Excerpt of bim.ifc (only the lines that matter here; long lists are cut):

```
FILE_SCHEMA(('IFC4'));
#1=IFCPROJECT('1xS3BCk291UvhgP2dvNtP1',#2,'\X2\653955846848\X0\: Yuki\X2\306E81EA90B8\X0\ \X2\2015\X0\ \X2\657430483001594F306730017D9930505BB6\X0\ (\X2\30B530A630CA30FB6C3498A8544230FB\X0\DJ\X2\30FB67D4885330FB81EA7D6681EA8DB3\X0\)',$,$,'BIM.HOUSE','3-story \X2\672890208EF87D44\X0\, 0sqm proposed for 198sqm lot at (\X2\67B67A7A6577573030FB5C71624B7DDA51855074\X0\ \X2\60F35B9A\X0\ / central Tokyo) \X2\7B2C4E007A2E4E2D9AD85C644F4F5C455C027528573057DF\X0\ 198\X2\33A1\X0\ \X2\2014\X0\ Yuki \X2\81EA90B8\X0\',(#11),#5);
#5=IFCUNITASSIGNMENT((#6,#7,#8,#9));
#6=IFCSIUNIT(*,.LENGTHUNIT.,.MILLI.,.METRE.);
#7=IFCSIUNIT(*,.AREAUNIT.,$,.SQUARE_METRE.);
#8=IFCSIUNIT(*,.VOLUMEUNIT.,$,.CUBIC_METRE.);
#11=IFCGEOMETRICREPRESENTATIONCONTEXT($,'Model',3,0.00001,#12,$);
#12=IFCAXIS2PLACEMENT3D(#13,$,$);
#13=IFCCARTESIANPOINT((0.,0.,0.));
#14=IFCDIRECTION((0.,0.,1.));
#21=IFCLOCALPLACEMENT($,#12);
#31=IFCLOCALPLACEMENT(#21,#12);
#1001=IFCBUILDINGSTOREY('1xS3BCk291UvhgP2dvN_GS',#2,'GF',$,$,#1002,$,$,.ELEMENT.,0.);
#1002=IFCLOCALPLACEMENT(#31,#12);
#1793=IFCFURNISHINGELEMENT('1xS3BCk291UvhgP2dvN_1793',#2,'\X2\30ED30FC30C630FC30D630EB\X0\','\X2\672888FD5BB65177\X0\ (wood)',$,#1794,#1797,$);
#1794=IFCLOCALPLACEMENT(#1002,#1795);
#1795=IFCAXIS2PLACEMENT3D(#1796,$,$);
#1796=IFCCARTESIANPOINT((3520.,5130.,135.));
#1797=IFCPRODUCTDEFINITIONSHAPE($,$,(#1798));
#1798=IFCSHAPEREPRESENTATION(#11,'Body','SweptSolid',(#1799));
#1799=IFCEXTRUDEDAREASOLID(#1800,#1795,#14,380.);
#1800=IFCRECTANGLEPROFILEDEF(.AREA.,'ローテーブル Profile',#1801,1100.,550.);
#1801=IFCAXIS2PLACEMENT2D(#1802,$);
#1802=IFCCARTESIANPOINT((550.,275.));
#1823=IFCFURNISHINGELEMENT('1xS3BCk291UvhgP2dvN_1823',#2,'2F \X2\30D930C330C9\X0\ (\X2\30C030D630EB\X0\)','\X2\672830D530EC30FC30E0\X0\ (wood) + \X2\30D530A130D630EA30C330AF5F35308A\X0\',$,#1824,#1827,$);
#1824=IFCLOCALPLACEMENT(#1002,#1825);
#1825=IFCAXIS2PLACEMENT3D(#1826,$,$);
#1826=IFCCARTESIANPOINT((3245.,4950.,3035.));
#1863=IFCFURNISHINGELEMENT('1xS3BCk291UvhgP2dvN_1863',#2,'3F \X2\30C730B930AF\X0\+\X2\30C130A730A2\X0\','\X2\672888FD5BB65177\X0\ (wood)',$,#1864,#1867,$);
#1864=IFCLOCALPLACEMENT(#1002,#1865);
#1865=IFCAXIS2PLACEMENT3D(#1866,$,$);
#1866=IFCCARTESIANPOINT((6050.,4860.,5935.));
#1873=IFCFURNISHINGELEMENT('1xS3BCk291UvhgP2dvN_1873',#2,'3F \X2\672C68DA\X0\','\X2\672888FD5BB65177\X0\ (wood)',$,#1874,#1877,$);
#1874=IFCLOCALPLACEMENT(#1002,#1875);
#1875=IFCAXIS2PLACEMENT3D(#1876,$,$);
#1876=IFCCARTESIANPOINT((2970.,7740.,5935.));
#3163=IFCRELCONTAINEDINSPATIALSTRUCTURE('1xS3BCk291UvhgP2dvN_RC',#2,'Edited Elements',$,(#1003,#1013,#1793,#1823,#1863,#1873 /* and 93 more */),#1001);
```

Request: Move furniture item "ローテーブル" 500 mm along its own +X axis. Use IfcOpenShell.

```python
import ifcopenshell
import ifcopenshell.api.geometry
import ifcopenshell.util.placement

model = ifcopenshell.open("bim.ifc")

item = model.by_id(1793)
matrix = ifcopenshell.util.placement.get_local_placement(item.ObjectPlacement)
matrix[:3, 3] += matrix[:3, 0] * 500.0
ifcopenshell.api.geometry.edit_object_placement(model, product=item, matrix=matrix, is_si=False)

print(ifcopenshell.util.placement.get_local_placement(item.ObjectPlacement).round(3) + 0.0)

model.write("bim-out.ifc")
```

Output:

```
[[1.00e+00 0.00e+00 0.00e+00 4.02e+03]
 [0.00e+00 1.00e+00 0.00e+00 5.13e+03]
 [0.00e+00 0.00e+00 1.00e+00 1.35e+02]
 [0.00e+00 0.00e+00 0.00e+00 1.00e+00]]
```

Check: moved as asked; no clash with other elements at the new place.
